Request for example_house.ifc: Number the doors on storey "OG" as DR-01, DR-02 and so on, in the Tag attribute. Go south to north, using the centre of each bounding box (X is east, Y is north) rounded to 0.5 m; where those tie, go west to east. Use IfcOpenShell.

First a look at what the model holds.

```python
import ifcopenshell
import ifcopenshell.util.element
import ifcopenshell.util.placement

model = ifcopenshell.open("example_house.ifc")
print(model.schema)
storey = next(s for s in model.by_type("IfcBuildingStorey") if s.Name == "OG")
doors = [e for e in ifcopenshell.util.element.get_decomposition(storey) if e.is_a("IfcDoor")]
for e in sorted(doors, key=lambda e: e.id()):
    origin = ifcopenshell.util.placement.get_local_placement(e.ObjectPlacement)[:3, 3]
    print(e.id(), e.Tag, e.Name, origin.round(2) + 0.0, sep=" | ")
```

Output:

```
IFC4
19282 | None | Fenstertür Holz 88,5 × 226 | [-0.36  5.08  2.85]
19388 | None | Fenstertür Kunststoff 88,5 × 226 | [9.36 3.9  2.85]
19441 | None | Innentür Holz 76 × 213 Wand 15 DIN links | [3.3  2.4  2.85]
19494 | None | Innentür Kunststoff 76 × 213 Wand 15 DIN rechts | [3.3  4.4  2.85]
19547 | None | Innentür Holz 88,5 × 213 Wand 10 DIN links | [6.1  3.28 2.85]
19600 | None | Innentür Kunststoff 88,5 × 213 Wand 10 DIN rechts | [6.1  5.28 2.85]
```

```python
import ifcopenshell
import ifcopenshell.geom
import ifcopenshell.util.element
import ifcopenshell.util.shape

model = ifcopenshell.open("example_house.ifc")
settings = ifcopenshell.geom.settings()
settings.set("use-world-coords", True)


def centre(element):
    shape = ifcopenshell.geom.create_shape(settings, element)
    return ifcopenshell.util.shape.get_bbox_centroid(shape.geometry)


storey = next(s for s in model.by_type("IfcBuildingStorey") if s.Name == "OG")
doors = [e for e in ifcopenshell.util.element.get_decomposition(storey) if e.is_a("IfcDoor")]

# Insertion points can sit at a corner or the storey origin, so sort by the geometry (in metres).
centres = {e: centre(e) for e in doors}
doors.sort(key=lambda e: (round(centres[e][1] / 0.5), centres[e][0]))

for i, e in enumerate(doors, start=1):
    number = f"DR-{i:02d}"
    e.Tag = number
    print(e.id(), number)

model.write("example_house_v2.ifc")
```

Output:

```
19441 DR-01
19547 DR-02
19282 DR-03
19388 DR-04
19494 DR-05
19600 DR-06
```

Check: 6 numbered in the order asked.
